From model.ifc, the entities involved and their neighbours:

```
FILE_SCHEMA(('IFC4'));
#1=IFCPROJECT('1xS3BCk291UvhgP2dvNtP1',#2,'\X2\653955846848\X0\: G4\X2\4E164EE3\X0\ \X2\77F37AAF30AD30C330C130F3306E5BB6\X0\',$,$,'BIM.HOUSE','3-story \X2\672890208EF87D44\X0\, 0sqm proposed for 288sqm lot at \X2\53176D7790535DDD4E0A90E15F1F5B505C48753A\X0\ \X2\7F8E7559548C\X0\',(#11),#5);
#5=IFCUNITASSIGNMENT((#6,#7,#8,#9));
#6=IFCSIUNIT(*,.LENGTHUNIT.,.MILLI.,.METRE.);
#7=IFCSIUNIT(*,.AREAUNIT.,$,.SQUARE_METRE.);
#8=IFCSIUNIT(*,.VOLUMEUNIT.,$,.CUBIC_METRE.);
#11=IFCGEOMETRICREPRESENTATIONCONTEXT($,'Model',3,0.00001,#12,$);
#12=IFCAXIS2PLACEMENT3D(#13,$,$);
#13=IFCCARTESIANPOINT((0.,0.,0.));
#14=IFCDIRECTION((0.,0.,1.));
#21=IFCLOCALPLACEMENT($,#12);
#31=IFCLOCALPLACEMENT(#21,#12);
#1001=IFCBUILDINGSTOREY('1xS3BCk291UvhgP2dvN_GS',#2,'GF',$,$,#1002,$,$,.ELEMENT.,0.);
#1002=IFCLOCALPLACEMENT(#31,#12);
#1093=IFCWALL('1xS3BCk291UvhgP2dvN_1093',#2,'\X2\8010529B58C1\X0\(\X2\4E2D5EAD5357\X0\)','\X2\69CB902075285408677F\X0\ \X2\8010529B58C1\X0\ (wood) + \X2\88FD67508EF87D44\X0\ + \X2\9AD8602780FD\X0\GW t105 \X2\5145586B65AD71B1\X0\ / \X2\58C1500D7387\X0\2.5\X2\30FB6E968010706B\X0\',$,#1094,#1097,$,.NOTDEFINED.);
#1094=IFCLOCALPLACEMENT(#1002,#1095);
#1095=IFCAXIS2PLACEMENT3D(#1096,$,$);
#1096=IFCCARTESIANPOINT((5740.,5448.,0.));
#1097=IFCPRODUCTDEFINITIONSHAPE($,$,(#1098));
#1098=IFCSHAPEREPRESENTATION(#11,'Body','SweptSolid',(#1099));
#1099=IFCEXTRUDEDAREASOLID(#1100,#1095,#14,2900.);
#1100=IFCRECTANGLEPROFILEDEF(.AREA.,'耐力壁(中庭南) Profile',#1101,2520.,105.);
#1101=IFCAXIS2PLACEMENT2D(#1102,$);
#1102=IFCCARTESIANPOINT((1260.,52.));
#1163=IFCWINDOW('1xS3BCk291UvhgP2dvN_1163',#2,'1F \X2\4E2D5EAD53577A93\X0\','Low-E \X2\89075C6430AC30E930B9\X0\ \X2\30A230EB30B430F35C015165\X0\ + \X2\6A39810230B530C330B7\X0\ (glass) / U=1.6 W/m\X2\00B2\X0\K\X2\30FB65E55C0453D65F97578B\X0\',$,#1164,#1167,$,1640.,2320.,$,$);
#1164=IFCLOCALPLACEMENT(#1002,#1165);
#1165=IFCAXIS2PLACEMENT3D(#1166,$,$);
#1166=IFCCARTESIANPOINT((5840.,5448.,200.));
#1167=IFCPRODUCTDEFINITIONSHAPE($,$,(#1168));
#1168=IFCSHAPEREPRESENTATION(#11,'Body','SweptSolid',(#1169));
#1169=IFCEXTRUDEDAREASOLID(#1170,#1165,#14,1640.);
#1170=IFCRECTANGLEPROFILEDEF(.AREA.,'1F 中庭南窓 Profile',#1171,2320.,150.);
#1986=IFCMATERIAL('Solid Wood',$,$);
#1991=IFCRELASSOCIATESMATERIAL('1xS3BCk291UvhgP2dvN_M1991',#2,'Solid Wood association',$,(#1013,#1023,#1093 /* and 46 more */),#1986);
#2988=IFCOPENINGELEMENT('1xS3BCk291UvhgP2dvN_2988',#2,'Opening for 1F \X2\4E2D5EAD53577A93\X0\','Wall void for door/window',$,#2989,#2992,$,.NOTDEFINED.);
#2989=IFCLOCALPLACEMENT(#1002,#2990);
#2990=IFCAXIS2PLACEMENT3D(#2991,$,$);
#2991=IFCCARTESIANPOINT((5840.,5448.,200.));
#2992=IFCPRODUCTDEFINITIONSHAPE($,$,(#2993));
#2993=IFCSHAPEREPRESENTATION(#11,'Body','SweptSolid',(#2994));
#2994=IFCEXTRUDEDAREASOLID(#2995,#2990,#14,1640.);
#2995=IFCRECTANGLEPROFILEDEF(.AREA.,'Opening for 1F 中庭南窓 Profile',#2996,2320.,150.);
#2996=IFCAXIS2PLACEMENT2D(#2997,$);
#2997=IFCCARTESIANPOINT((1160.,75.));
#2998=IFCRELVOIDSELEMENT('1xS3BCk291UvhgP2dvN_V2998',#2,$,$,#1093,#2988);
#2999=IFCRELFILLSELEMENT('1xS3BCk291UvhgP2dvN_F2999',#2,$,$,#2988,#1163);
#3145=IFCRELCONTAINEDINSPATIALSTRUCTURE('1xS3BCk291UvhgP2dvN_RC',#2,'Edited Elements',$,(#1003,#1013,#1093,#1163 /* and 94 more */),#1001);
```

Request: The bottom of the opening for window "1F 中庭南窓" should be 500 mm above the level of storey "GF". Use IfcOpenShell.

```python
import numpy as np
import ifcopenshell
import ifcopenshell.api.geometry
import ifcopenshell.geom
import ifcopenshell.util.element
import ifcopenshell.util.placement
import ifcopenshell.util.shape
import ifcopenshell.util.unit

model = ifcopenshell.open("model.ifc")
unit_scale = ifcopenshell.util.unit.calculate_unit_scale(model)

window = model.by_guid("1xS3BCk291UvhgP2dvN_1163")
opening = window.FillsVoids[0].RelatingOpeningElement
storey = ifcopenshell.util.element.get_container(window, ifc_class="IfcBuildingStorey")
level = ifcopenshell.util.placement.get_local_placement(storey.ObjectPlacement)[2, 3]

# The opening's origin need not be at the sill, so measure its lowest point.
shape = ifcopenshell.geom.create_shape(ifcopenshell.geom.settings(), opening)
bottom = ifcopenshell.util.shape.get_shape_bottom_elevation(shape, shape.geometry) / unit_scale
dz = level + 0.5 / unit_scale - bottom

shift = np.array([0.0, 0.0, dz])
# The window is not placed relative to its opening, so move both.
for product in (opening, window):
    matrix = ifcopenshell.util.placement.get_local_placement(product.ObjectPlacement)
    matrix[:3, 3] += shift
    ifcopenshell.api.geometry.edit_object_placement(model, product=product, matrix=matrix, is_si=False)

print(f"moved by {dz * unit_scale:+.3f} m")

model.write("model_v2.ifc")
```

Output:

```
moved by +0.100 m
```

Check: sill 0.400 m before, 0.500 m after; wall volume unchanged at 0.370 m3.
